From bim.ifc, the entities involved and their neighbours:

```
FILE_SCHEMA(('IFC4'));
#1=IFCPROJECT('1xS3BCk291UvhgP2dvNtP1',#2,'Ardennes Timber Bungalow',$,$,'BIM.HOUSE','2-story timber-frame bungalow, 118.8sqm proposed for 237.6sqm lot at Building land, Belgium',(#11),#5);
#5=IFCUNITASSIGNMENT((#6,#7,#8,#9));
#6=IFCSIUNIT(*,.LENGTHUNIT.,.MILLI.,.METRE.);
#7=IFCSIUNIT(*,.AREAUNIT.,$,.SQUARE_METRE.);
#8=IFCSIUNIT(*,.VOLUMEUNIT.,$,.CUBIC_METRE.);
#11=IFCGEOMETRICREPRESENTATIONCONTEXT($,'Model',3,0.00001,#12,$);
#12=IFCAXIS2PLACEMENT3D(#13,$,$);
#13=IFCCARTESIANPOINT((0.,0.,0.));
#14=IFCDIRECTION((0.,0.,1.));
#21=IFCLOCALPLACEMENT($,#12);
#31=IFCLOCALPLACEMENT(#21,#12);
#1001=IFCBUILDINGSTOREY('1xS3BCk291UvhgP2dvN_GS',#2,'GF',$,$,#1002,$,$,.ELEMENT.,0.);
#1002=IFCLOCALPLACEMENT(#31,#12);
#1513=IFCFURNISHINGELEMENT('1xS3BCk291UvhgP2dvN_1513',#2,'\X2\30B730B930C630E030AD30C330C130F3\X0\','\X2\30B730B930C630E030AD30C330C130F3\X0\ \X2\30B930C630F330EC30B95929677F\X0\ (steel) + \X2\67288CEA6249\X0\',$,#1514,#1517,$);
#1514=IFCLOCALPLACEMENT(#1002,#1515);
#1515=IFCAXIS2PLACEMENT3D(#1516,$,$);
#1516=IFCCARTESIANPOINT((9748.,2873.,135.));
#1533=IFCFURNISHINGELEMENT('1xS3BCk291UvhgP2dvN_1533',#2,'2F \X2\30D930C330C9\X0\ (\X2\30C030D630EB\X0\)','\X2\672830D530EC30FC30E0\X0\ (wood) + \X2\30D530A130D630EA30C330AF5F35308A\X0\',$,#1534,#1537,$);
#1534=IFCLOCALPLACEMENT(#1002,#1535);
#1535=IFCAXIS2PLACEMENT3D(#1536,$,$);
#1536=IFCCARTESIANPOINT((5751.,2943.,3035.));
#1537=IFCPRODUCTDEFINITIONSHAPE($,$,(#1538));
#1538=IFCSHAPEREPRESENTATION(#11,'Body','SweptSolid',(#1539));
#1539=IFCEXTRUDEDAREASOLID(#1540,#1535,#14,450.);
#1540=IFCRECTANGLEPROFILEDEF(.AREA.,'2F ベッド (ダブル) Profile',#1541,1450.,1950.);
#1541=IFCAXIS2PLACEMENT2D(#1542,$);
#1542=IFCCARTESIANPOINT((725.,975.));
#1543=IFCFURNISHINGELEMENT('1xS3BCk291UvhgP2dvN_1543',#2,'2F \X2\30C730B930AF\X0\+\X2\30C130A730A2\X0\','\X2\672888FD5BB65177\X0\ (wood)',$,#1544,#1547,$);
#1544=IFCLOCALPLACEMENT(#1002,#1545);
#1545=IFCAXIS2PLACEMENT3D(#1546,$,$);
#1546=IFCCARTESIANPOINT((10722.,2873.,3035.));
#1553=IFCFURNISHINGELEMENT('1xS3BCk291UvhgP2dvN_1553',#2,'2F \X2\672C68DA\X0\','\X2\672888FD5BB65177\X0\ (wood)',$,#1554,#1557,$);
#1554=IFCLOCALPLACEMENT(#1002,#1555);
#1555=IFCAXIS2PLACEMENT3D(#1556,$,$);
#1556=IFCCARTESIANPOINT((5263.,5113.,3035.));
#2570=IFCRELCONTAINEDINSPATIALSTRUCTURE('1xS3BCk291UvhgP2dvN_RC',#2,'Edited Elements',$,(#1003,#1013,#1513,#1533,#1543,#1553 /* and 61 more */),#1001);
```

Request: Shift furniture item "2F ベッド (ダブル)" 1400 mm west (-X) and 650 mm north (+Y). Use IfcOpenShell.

```python
import ifcopenshell
import ifcopenshell.api.geometry
import ifcopenshell.util.placement
import ifcopenshell.util.unit

model = ifcopenshell.open("bim.ifc")
unit_scale = ifcopenshell.util.unit.calculate_unit_scale(model)

item = model.by_guid("1xS3BCk291UvhgP2dvN_1533")
matrix = ifcopenshell.util.placement.get_local_placement(item.ObjectPlacement)
matrix[0, 3] -= 1.4 / unit_scale
matrix[1, 3] += 0.65 / unit_scale
ifcopenshell.api.geometry.edit_object_placement(model, product=item, matrix=matrix, is_si=False)

print(ifcopenshell.util.placement.get_local_placement(item.ObjectPlacement).round(3) + 0.0)

model.write("bim_rev.ifc")
```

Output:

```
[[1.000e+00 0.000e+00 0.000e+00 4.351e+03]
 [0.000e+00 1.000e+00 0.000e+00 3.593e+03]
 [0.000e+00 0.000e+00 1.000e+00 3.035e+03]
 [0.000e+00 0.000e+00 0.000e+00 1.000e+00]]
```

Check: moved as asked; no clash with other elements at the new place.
